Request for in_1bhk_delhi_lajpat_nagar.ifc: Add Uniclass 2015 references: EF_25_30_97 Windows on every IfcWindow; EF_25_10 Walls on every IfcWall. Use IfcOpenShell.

First a look at what the model holds.

```python
import ifcopenshell

model = ifcopenshell.open("in_1bhk_delhi_lajpat_nagar.ifc")
print(model.schema)
print("classifications:", [c.Name for c in model.by_type("IfcClassification")])
for ifc_class in ("IfcDoor", "IfcRoof", "IfcStair", "IfcWall", "IfcWindow"):
    print(ifc_class, len(model.by_type(ifc_class)))
```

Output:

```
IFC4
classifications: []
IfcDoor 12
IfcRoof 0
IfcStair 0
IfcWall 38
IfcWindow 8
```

```python
import ifcopenshell
import ifcopenshell.api.classification

model = ifcopenshell.open("in_1bhk_delhi_lajpat_nagar.ifc")

system = ifcopenshell.api.classification.add_classification(model, classification="Uniclass 2015")

codes = {
    "IfcWindow": ("EF_25_30_97", "Windows"),
    "IfcWall": ("EF_25_10", "Walls"),
}
for ifc_class, (code, name) in codes.items():
    products = model.by_type(ifc_class)
    ifcopenshell.api.classification.add_reference(
        model, products=products, classification=system, identification=code, name=name
    )
    print(code, len(products))

model.write("in_1bhk_delhi_lajpat_nagar_edited.ifc")
```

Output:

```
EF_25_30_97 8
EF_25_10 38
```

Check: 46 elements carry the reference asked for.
